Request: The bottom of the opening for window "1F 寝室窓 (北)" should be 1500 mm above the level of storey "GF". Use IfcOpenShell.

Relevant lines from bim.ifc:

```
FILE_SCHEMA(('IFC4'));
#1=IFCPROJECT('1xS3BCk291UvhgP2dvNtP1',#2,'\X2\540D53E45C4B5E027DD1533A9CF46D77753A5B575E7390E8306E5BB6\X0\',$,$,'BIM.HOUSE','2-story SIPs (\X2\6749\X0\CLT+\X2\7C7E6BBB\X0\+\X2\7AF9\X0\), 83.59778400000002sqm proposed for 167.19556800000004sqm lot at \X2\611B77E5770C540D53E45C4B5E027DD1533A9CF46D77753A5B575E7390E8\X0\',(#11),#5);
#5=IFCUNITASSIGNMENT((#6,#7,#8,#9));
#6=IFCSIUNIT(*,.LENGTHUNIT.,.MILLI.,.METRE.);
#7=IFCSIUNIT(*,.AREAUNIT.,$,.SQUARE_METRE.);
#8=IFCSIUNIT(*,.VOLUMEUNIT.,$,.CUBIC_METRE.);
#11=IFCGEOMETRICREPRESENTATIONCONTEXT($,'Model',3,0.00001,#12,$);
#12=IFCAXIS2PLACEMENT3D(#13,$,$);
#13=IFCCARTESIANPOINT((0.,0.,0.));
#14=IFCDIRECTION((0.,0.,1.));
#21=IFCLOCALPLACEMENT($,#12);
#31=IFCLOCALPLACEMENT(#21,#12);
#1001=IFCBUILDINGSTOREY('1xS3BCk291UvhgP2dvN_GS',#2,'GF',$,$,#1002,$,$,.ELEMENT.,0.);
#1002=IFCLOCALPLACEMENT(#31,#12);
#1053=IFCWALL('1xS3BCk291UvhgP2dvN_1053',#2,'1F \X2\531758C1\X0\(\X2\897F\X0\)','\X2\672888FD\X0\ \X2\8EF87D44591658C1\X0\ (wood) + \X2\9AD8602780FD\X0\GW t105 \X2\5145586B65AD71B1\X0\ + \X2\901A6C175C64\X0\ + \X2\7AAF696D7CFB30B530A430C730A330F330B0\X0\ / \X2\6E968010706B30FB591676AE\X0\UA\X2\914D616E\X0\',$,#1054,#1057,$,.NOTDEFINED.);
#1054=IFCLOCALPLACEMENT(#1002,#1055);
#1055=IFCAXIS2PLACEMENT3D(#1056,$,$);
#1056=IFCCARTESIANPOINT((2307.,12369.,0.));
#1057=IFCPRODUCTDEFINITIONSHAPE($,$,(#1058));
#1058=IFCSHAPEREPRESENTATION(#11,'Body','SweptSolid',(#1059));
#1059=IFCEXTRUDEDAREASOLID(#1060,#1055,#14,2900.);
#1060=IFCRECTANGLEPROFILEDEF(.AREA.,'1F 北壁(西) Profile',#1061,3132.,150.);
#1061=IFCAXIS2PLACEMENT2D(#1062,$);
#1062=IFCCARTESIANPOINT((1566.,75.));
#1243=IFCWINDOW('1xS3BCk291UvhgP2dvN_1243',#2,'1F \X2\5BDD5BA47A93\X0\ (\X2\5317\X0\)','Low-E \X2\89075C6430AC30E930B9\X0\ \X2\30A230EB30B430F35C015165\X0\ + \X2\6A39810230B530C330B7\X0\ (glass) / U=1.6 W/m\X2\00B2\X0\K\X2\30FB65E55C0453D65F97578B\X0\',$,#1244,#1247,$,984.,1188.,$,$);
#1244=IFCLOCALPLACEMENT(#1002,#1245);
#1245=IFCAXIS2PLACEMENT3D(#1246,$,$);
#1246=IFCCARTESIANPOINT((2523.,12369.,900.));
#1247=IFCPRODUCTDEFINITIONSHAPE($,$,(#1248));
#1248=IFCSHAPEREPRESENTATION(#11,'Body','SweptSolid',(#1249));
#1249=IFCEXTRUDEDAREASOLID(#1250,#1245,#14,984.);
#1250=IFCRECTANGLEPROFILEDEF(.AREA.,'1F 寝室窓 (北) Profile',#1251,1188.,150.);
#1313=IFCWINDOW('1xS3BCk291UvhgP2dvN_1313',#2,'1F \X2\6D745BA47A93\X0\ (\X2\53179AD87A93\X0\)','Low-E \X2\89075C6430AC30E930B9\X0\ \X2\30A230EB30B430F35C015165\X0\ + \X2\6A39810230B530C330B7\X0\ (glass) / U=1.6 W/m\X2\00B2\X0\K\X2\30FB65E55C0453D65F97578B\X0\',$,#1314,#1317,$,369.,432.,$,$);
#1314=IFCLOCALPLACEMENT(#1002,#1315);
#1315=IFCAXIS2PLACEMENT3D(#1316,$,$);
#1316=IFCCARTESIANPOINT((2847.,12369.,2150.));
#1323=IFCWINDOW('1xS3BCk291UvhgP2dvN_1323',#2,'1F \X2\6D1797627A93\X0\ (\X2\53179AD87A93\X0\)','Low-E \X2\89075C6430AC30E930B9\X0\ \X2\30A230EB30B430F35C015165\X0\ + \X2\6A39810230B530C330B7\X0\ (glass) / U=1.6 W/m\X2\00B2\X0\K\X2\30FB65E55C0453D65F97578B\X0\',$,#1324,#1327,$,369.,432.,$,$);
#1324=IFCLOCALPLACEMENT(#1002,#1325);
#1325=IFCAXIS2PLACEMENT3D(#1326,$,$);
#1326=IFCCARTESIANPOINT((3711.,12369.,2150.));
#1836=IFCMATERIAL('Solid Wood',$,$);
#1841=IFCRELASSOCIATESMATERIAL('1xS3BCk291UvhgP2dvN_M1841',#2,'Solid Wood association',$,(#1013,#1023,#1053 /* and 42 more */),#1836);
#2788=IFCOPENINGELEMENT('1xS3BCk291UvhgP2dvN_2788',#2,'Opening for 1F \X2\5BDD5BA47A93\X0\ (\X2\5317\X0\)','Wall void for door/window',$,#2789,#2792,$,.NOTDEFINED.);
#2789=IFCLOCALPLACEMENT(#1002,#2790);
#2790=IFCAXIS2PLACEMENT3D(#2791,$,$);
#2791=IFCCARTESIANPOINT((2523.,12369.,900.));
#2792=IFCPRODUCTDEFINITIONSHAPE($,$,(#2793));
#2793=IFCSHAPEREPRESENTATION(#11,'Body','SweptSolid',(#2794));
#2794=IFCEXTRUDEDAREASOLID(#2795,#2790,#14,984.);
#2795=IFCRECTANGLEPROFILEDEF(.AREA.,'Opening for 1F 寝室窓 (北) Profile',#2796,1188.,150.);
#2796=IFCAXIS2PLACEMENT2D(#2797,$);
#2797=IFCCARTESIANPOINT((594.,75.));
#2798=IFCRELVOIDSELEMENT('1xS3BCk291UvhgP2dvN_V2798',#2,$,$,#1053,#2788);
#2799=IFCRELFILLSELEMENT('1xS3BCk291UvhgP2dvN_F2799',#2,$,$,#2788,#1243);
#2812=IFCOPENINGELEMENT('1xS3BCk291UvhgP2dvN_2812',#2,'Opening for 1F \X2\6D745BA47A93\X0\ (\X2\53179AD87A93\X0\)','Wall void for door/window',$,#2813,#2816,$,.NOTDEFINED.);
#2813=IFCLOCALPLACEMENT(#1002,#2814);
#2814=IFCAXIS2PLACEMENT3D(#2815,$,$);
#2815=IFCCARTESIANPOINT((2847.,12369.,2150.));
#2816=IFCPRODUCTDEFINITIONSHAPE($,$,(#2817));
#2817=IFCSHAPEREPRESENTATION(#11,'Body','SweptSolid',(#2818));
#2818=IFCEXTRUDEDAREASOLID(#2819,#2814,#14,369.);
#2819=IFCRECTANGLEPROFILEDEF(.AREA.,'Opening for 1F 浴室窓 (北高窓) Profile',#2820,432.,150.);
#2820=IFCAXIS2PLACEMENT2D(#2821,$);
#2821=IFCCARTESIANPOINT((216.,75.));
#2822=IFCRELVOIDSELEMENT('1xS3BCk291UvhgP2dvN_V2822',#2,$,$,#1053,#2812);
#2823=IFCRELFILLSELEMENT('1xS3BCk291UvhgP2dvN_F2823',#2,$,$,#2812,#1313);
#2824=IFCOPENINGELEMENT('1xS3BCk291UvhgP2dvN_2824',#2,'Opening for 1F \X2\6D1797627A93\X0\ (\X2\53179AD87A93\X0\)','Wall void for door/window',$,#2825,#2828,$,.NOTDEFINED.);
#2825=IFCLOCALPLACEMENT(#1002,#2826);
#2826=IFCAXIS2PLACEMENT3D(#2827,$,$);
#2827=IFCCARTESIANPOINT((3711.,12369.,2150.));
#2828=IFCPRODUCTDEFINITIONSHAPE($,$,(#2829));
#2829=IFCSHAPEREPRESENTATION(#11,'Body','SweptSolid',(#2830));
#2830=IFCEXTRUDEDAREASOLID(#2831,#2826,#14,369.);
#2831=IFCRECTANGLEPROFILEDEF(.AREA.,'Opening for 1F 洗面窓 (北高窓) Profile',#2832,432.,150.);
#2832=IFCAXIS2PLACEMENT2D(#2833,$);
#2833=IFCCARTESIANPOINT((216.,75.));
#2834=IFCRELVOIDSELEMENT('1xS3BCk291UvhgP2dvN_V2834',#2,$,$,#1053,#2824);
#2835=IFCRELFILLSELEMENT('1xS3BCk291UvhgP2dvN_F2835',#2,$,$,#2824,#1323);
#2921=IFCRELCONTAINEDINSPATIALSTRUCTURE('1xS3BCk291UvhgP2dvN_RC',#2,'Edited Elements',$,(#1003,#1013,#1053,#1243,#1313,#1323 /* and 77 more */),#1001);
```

```python
import numpy as np
import ifcopenshell
import ifcopenshell.api.geometry
import ifcopenshell.geom
import ifcopenshell.util.element
import ifcopenshell.util.placement
import ifcopenshell.util.shape
import ifcopenshell.util.unit

model = ifcopenshell.open("bim.ifc")
unit_scale = ifcopenshell.util.unit.calculate_unit_scale(model)

window = model.by_guid("1xS3BCk291UvhgP2dvN_1243")
opening = window.FillsVoids[0].RelatingOpeningElement
storey = ifcopenshell.util.element.get_container(window, ifc_class="IfcBuildingStorey")
level = ifcopenshell.util.placement.get_local_placement(storey.ObjectPlacement)[2, 3]

# The opening's origin need not be at the sill, so measure its lowest point.
shape = ifcopenshell.geom.create_shape(ifcopenshell.geom.settings(), opening)
bottom = ifcopenshell.util.shape.get_shape_bottom_elevation(shape, shape.geometry) / unit_scale
dz = level + 1.5 / unit_scale - bottom

shift = np.array([0.0, 0.0, dz])
# The window is not placed relative to its opening, so move both.
for product in (opening, window):
    matrix = ifcopenshell.util.placement.get_local_placement(product.ObjectPlacement)
    matrix[:3, 3] += shift
    ifcopenshell.api.geometry.edit_object_placement(model, product=product, matrix=matrix, is_si=False)

print(f"moved by {dz * unit_scale:+.3f} m")

model.write("bim_edited.ifc")
```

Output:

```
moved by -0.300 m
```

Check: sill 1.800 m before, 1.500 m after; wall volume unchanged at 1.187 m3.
